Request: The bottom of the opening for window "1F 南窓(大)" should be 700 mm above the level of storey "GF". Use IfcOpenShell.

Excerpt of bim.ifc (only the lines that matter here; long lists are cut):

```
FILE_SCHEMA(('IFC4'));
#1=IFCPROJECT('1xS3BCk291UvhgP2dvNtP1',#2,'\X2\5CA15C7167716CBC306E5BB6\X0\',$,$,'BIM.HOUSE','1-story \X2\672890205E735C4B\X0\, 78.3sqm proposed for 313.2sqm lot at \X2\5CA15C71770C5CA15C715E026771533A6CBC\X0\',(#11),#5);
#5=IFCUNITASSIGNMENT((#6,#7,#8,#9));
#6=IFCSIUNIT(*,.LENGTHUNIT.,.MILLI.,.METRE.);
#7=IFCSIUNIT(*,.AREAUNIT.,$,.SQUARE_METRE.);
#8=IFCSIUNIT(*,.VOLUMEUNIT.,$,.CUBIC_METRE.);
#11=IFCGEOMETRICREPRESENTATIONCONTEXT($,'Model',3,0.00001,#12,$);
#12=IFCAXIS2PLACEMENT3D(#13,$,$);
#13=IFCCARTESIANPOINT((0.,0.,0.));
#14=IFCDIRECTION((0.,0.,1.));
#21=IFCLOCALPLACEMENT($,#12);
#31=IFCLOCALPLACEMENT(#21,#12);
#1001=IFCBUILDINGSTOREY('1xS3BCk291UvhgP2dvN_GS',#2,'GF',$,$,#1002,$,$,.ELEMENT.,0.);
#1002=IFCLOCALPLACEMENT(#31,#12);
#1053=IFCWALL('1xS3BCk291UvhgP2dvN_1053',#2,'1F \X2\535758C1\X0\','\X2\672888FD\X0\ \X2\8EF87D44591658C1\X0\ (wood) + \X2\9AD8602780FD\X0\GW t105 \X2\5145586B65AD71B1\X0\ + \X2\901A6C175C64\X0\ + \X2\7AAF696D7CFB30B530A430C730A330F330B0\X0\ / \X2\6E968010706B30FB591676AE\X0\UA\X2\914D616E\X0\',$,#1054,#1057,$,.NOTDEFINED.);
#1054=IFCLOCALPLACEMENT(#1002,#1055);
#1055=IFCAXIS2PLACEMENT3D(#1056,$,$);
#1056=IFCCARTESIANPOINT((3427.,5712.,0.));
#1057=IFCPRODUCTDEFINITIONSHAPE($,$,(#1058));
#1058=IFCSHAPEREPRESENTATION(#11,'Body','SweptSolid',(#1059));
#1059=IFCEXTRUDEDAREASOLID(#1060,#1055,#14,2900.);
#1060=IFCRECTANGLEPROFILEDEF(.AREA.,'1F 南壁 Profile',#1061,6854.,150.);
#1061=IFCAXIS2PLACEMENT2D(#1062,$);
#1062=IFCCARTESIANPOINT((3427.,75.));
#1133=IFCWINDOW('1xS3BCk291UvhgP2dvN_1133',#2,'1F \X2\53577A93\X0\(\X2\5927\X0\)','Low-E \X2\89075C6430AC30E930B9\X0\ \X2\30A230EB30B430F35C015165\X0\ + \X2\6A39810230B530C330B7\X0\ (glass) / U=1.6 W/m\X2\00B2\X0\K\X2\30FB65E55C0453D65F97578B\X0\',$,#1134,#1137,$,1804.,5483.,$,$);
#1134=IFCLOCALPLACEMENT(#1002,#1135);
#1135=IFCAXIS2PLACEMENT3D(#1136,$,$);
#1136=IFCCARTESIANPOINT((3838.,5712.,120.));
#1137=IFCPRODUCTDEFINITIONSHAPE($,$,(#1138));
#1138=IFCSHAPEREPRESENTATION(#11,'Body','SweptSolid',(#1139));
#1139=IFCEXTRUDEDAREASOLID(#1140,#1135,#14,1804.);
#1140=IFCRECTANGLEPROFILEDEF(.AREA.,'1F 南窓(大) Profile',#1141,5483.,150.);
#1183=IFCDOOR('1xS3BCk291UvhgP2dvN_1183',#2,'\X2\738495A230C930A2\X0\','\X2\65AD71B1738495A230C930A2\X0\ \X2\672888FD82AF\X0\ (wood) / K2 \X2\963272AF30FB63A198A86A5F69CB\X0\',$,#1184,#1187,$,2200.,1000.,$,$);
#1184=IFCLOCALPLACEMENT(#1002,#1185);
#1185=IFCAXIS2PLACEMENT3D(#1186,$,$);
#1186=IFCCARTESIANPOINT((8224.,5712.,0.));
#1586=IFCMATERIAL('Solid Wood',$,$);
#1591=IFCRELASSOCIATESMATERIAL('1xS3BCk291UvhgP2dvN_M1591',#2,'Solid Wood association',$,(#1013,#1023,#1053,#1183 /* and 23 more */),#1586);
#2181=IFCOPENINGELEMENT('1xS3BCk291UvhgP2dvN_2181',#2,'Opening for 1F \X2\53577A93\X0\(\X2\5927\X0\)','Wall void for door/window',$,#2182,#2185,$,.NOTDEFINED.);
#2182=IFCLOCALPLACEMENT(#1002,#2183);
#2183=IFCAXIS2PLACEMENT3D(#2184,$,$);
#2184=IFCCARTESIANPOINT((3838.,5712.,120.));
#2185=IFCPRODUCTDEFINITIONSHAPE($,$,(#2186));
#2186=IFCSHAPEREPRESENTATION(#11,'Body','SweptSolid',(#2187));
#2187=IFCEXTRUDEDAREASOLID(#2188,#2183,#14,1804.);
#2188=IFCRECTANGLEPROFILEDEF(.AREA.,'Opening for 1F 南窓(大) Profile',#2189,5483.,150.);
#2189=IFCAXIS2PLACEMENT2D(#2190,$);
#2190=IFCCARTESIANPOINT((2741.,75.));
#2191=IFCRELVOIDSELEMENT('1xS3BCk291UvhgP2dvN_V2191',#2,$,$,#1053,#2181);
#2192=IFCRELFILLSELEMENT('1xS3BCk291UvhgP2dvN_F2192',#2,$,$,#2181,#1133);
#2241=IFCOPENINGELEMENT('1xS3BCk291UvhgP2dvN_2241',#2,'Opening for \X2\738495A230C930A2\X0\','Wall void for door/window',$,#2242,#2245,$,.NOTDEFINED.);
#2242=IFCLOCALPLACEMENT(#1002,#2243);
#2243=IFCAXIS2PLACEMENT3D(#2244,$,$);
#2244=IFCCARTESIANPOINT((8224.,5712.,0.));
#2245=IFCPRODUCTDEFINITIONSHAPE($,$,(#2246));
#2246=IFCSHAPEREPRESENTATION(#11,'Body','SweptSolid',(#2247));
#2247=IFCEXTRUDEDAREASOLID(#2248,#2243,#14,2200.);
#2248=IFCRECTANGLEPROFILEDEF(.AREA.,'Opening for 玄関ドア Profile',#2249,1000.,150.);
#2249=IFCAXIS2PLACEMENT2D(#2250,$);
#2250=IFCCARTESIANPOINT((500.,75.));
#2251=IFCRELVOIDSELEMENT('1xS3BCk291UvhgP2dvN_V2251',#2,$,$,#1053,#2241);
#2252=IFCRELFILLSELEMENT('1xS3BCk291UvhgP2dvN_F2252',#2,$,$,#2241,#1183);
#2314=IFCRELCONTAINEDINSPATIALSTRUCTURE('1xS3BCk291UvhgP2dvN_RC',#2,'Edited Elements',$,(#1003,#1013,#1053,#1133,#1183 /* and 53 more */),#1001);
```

```python
import numpy as np
import ifcopenshell
import ifcopenshell.api.geometry
import ifcopenshell.geom
import ifcopenshell.util.element
import ifcopenshell.util.placement
import ifcopenshell.util.shape
import ifcopenshell.util.unit

model = ifcopenshell.open("bim.ifc")
unit_scale = ifcopenshell.util.unit.calculate_unit_scale(model)

window = model.by_id(1133)
opening = window.FillsVoids[0].RelatingOpeningElement
storey = ifcopenshell.util.element.get_container(window, ifc_class="IfcBuildingStorey")
level = ifcopenshell.util.placement.get_local_placement(storey.ObjectPlacement)[2, 3]

# The opening's origin need not be at the sill, so measure its lowest point.
shape = ifcopenshell.geom.create_shape(ifcopenshell.geom.settings(), opening)
bottom = ifcopenshell.util.shape.get_shape_bottom_elevation(shape, shape.geometry) / unit_scale
dz = level + 0.7 / unit_scale - bottom

shift = np.array([0.0, 0.0, dz])
# The window is not placed relative to its opening, so move both.
for product in (opening, window):
    matrix = ifcopenshell.util.placement.get_local_placement(product.ObjectPlacement)
    matrix[:3, 3] += shift
    ifcopenshell.api.geometry.edit_object_placement(model, product=product, matrix=matrix, is_si=False)

print(f"moved by {dz * unit_scale:+.3f} m")

model.write("bim_edited.ifc")
```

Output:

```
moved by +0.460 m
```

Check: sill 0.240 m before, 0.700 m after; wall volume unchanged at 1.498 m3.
